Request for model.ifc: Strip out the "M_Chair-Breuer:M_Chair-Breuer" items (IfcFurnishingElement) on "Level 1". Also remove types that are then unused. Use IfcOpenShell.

First a look at what the model holds.

```python
import ifcopenshell
import ifcopenshell.util.element

model = ifcopenshell.open("model.ifc")
print(model.schema)
storey = next(s for s in model.by_type("IfcBuildingStorey") if s.Name == "Level 1")
furniture = [e for e in ifcopenshell.util.element.get_decomposition(storey) if e.is_a("IfcFurnishingElement")]
seen = {}
for e in furniture:
    element_type = ifcopenshell.util.element.get_type(e)
    name = element_type.Name if element_type not in (None, e) else None
    seen[name] = seen.get(name, 0) + 1
for name, count in sorted(seen.items(), key=str):
    print(count, "x", name)
```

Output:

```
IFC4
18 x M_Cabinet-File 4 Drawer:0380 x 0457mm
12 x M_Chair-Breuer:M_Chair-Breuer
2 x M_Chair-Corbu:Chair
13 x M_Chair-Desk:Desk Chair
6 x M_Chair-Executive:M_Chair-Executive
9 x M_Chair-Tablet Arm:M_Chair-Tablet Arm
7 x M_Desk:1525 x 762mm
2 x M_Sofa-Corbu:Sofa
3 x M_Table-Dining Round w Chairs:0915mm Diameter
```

```python
import ifcopenshell
import ifcopenshell.api.root
import ifcopenshell.util.element

model = ifcopenshell.open("model.ifc")

storey = next(s for s in model.by_type("IfcBuildingStorey") if s.Name == "Level 1")
furniture = [e for e in ifcopenshell.util.element.get_decomposition(storey) if e.is_a("IfcFurnishingElement")]
targets = [e for e in furniture if (t := ifcopenshell.util.element.get_type(e)) not in (None, e) and t.Name == "M_Chair-Breuer:M_Chair-Breuer"]
types = {ifcopenshell.util.element.get_type(e) for e in targets} - {None, *targets}

for e in targets:
    ifcopenshell.api.root.remove_product(model, product=e)
print(len(targets), "removed")

unused = [t for t in types if not ifcopenshell.util.element.get_types(t)]
for t in unused:
    ifcopenshell.api.root.remove_product(model, product=t)
print(len(unused), "unused types removed")

model.write("model_rev.ifc")
```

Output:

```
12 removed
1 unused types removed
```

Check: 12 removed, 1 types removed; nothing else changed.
